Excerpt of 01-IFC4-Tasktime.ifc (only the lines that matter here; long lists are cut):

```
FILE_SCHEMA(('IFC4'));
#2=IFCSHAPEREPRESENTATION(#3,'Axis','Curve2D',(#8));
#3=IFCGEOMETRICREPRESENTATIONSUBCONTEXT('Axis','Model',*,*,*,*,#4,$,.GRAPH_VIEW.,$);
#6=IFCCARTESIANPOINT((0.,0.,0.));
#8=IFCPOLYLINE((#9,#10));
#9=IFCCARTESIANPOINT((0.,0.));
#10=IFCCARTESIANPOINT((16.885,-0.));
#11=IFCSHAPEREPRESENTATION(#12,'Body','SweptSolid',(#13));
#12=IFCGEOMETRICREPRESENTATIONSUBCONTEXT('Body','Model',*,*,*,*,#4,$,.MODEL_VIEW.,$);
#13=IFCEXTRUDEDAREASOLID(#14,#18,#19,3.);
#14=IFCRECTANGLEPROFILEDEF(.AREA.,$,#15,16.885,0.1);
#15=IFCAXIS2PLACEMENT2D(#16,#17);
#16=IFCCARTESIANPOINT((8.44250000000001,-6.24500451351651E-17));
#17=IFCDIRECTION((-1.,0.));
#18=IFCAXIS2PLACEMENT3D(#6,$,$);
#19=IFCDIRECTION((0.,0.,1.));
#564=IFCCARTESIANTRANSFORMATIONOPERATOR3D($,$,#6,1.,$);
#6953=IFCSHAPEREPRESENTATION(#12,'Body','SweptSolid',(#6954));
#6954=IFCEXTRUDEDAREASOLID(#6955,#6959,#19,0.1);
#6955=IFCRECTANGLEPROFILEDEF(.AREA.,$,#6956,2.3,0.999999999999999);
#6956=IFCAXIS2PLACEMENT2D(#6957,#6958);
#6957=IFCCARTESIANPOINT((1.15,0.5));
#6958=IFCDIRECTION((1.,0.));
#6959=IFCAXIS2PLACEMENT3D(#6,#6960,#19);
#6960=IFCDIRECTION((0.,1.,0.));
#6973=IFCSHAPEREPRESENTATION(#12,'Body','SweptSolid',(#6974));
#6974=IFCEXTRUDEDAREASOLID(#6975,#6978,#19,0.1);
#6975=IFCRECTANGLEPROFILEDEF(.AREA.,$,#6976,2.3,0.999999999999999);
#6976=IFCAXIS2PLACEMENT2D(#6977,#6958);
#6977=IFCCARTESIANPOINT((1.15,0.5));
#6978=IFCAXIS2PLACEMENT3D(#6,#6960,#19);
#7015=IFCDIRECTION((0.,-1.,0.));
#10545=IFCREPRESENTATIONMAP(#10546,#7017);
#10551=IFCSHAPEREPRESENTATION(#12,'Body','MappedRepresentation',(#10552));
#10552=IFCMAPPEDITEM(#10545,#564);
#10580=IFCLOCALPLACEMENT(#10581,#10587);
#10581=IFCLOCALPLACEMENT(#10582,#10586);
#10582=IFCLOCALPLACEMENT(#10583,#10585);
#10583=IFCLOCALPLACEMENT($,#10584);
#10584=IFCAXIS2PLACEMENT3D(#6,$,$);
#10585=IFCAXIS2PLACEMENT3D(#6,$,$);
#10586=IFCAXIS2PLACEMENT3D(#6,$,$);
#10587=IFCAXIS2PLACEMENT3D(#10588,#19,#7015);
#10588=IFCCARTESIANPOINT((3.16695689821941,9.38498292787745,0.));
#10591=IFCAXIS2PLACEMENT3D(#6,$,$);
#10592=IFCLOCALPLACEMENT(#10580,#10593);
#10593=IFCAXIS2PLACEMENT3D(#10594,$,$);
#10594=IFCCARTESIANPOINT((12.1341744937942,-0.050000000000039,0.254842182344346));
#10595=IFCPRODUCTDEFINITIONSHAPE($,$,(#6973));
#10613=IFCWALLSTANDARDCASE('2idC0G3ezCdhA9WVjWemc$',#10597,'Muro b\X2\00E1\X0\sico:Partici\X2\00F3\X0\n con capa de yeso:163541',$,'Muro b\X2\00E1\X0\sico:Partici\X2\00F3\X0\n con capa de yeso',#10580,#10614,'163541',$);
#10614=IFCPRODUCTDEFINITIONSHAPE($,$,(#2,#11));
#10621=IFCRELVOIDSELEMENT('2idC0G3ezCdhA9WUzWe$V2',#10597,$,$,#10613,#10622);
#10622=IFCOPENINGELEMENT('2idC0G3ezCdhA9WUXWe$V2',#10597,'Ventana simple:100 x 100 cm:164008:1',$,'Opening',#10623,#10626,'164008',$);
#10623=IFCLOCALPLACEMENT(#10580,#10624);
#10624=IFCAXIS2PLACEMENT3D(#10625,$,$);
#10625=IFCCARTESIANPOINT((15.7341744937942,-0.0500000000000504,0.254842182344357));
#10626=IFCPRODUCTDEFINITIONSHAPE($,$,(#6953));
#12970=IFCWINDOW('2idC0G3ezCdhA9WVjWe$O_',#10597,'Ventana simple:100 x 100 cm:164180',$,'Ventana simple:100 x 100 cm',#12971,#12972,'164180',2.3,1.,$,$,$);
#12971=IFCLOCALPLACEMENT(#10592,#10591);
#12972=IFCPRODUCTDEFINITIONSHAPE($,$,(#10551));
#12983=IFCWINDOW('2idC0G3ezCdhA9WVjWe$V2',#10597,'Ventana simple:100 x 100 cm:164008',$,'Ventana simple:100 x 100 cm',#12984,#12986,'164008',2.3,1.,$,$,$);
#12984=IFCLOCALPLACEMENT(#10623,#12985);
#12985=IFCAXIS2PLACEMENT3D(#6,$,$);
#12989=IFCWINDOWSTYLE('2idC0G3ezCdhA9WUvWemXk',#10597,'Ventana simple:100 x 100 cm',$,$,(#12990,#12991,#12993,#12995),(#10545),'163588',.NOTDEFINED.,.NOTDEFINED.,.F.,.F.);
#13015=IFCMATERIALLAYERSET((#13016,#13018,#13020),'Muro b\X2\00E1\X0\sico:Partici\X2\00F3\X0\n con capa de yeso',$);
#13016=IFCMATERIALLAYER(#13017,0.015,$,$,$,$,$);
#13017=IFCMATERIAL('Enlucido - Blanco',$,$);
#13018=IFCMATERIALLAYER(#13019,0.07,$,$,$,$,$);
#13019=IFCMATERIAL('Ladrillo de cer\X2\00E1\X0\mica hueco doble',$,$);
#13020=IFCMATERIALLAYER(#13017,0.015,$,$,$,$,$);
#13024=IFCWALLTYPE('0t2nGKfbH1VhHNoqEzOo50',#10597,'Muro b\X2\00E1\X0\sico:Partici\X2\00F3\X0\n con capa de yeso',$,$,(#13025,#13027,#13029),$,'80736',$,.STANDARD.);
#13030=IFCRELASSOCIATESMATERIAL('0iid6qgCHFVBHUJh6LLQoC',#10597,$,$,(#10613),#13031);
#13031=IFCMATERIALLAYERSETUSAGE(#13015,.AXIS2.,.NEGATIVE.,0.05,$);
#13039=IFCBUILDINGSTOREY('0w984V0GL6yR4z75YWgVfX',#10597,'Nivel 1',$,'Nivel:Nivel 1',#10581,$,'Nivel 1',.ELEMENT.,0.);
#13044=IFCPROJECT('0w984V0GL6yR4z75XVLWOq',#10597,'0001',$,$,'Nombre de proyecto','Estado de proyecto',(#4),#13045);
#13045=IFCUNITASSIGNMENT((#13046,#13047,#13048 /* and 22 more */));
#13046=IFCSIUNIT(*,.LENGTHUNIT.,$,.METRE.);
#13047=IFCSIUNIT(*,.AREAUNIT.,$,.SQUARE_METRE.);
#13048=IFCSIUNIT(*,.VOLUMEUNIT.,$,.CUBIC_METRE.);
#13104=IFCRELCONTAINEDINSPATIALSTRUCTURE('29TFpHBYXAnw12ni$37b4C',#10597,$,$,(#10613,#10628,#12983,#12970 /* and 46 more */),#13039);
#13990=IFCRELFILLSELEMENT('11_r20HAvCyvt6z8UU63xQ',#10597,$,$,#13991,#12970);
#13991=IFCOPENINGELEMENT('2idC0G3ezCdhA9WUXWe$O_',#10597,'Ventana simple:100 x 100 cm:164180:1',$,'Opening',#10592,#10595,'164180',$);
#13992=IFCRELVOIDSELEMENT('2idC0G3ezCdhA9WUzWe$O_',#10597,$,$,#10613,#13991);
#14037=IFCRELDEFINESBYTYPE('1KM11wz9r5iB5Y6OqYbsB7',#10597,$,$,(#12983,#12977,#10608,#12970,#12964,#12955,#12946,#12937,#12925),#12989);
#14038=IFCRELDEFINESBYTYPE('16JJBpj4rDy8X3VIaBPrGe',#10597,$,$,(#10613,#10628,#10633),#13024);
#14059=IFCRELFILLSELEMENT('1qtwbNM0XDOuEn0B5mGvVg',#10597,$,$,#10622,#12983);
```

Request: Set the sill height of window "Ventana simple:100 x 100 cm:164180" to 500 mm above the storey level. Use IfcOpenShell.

```python
import numpy as np
import ifcopenshell
import ifcopenshell.api.geometry
import ifcopenshell.geom
import ifcopenshell.util.element
import ifcopenshell.util.placement
import ifcopenshell.util.shape
import ifcopenshell.util.unit

model = ifcopenshell.open("01-IFC4-Tasktime.ifc")
unit_scale = ifcopenshell.util.unit.calculate_unit_scale(model)

window = model.by_guid("2idC0G3ezCdhA9WVjWe$O_")
opening = window.FillsVoids[0].RelatingOpeningElement
storey = ifcopenshell.util.element.get_container(window, ifc_class="IfcBuildingStorey")
level = ifcopenshell.util.placement.get_local_placement(storey.ObjectPlacement)[2, 3]

# The opening's origin need not be at the sill, so measure its lowest point.
shape = ifcopenshell.geom.create_shape(ifcopenshell.geom.settings(), opening)
bottom = ifcopenshell.util.shape.get_shape_bottom_elevation(shape, shape.geometry) / unit_scale
dz = level + 0.5 - bottom

shift = np.array([0.0, 0.0, dz])
# The window is placed relative to its opening, so it follows when the opening moves.
matrix = ifcopenshell.util.placement.get_local_placement(opening.ObjectPlacement)
matrix[:3, 3] += shift
ifcopenshell.api.geometry.edit_object_placement(
    model, product=opening, matrix=matrix, is_si=False, should_transform_children=True
)

print(f"moved by {dz * unit_scale:+.3f} m")

model.write("01-IFC4-Tasktime_updated.ifc")
```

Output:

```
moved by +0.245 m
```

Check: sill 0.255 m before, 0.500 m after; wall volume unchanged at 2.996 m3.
